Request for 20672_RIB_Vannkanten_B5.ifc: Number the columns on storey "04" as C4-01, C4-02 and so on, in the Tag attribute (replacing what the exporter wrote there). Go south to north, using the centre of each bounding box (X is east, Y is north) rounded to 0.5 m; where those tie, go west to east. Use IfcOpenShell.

First a look at what the model holds.

```python
import ifcopenshell
import ifcopenshell.util.element
import ifcopenshell.util.placement

model = ifcopenshell.open("20672_RIB_Vannkanten_B5.ifc")
print(model.schema)
storey = next(s for s in model.by_type("IfcBuildingStorey") if s.Name == "04")
columns = [e for e in ifcopenshell.util.element.get_decomposition(storey) if e.is_a("IfcColumn")]
for e in sorted(columns, key=lambda e: e.id()):
    origin = ifcopenshell.util.placement.get_local_placement(e.ObjectPlacement)[:3, 3]
    print(e.id(), e.Tag, e.Name, origin.round(2) + 0.0, sep=" | ")
```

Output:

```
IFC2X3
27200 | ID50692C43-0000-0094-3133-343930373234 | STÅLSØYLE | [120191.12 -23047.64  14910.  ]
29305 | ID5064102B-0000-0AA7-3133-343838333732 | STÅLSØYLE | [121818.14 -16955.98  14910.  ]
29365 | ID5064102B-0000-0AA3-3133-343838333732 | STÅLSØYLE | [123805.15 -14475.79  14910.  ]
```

```python
import ifcopenshell
import ifcopenshell.geom
import ifcopenshell.util.element
import ifcopenshell.util.shape

model = ifcopenshell.open("20672_RIB_Vannkanten_B5.ifc")
settings = ifcopenshell.geom.settings()
settings.set("use-world-coords", True)


def centre(element):
    shape = ifcopenshell.geom.create_shape(settings, element)
    return ifcopenshell.util.shape.get_bbox_centroid(shape.geometry)


storey = next(s for s in model.by_type("IfcBuildingStorey") if s.Name == "04")
columns = [e for e in ifcopenshell.util.element.get_decomposition(storey) if e.is_a("IfcColumn")]

# Insertion points can sit at a corner or the storey origin, so sort by the geometry (in metres).
centres = {e: centre(e) for e in columns}
columns.sort(key=lambda e: (round(centres[e][1] / 0.5), centres[e][0]))

for i, e in enumerate(columns, start=1):
    number = f"C4-{i:02d}"
    e.Tag = number
    print(e.id(), number)

model.write("20672_RIB_Vannkanten_B5-out.ifc")
```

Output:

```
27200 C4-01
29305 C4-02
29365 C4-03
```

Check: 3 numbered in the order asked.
